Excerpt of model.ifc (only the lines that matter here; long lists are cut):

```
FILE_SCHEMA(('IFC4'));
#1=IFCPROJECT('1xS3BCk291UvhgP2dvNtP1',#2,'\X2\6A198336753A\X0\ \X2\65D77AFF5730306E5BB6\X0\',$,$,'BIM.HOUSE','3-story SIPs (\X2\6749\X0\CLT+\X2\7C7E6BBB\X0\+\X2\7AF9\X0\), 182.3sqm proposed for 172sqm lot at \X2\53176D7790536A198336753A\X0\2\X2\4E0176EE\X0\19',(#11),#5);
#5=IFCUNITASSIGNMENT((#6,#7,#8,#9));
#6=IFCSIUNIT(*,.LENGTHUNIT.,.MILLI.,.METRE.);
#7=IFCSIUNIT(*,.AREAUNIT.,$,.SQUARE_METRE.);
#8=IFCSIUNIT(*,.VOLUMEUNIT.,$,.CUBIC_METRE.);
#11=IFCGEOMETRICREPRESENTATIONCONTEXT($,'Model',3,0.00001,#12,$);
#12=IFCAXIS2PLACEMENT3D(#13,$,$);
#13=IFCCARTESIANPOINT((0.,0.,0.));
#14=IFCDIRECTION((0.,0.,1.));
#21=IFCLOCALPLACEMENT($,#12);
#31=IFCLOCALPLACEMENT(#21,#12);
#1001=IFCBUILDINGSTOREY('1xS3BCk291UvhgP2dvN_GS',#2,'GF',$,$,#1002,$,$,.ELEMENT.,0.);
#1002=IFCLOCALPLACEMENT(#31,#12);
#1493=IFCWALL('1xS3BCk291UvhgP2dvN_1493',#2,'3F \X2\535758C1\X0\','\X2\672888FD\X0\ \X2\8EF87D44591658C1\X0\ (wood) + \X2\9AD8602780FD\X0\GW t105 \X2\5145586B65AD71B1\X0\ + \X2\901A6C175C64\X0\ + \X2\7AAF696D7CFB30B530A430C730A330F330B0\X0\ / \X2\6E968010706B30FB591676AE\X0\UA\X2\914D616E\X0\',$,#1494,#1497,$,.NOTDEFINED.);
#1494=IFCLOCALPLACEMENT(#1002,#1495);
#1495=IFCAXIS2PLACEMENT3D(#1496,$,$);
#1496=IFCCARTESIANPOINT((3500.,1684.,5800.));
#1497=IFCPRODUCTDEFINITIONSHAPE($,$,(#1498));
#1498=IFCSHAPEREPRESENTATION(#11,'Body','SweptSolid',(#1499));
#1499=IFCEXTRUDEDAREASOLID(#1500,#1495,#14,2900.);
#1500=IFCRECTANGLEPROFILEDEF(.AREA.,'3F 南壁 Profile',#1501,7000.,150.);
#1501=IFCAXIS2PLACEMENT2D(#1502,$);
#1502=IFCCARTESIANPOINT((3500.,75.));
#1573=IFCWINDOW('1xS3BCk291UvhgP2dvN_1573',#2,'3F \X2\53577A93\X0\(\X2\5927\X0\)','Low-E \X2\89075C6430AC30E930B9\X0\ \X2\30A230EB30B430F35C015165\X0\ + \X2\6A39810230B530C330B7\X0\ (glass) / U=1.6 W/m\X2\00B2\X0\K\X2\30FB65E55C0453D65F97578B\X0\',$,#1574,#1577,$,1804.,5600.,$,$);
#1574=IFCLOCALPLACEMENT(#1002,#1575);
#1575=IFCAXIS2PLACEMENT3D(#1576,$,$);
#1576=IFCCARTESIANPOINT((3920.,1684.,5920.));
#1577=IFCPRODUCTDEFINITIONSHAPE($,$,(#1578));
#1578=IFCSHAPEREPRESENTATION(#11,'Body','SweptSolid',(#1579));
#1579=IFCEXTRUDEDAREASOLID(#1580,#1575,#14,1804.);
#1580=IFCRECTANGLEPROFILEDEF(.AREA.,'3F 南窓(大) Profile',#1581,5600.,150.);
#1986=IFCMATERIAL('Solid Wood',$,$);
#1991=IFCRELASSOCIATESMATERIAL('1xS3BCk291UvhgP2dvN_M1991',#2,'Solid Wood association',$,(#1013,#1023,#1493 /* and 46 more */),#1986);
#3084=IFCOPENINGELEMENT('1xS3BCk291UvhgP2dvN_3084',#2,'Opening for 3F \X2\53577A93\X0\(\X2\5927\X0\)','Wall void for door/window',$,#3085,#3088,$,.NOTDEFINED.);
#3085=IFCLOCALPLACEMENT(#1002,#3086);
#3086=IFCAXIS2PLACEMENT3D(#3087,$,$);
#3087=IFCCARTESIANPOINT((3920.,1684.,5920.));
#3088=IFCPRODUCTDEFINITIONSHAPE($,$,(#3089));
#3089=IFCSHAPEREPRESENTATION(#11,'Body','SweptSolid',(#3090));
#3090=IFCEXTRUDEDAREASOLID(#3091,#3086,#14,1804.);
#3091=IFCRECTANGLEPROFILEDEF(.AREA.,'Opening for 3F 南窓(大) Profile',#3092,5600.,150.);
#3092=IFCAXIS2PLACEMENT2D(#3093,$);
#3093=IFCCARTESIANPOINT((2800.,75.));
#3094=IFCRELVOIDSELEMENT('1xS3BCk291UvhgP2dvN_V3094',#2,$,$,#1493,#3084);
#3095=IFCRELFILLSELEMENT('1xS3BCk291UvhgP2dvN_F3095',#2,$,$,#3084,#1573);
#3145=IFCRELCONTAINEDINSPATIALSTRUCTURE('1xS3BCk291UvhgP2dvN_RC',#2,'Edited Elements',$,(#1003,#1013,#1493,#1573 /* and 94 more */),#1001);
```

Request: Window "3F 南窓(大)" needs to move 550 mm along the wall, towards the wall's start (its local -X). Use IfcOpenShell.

```python
import ifcopenshell
import ifcopenshell.api.geometry
import ifcopenshell.util.placement
import ifcopenshell.util.unit

model = ifcopenshell.open("model.ifc")
unit_scale = ifcopenshell.util.unit.calculate_unit_scale(model)

window = model.by_guid("1xS3BCk291UvhgP2dvN_1573")
opening = window.FillsVoids[0].RelatingOpeningElement
wall = opening.VoidsElements[0].RelatingBuildingElement

wall_matrix = ifcopenshell.util.placement.get_local_placement(wall.ObjectPlacement)
shift = wall_matrix[:3, 0] * -0.55 / unit_scale
before = ifcopenshell.util.placement.get_local_placement(window.ObjectPlacement)[:3, 3].copy()

# The window is not placed relative to its opening, so move both.
for product in (opening, window):
    matrix = ifcopenshell.util.placement.get_local_placement(product.ObjectPlacement)
    matrix[:3, 3] += shift
    ifcopenshell.api.geometry.edit_object_placement(model, product=product, matrix=matrix, is_si=False)

after = ifcopenshell.util.placement.get_local_placement(window.ObjectPlacement)[:3, 3]
print("window moved by", (after - before).round(3) + 0.0)

model.write("model_edited.ifc")
```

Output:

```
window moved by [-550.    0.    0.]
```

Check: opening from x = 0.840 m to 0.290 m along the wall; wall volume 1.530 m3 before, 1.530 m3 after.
